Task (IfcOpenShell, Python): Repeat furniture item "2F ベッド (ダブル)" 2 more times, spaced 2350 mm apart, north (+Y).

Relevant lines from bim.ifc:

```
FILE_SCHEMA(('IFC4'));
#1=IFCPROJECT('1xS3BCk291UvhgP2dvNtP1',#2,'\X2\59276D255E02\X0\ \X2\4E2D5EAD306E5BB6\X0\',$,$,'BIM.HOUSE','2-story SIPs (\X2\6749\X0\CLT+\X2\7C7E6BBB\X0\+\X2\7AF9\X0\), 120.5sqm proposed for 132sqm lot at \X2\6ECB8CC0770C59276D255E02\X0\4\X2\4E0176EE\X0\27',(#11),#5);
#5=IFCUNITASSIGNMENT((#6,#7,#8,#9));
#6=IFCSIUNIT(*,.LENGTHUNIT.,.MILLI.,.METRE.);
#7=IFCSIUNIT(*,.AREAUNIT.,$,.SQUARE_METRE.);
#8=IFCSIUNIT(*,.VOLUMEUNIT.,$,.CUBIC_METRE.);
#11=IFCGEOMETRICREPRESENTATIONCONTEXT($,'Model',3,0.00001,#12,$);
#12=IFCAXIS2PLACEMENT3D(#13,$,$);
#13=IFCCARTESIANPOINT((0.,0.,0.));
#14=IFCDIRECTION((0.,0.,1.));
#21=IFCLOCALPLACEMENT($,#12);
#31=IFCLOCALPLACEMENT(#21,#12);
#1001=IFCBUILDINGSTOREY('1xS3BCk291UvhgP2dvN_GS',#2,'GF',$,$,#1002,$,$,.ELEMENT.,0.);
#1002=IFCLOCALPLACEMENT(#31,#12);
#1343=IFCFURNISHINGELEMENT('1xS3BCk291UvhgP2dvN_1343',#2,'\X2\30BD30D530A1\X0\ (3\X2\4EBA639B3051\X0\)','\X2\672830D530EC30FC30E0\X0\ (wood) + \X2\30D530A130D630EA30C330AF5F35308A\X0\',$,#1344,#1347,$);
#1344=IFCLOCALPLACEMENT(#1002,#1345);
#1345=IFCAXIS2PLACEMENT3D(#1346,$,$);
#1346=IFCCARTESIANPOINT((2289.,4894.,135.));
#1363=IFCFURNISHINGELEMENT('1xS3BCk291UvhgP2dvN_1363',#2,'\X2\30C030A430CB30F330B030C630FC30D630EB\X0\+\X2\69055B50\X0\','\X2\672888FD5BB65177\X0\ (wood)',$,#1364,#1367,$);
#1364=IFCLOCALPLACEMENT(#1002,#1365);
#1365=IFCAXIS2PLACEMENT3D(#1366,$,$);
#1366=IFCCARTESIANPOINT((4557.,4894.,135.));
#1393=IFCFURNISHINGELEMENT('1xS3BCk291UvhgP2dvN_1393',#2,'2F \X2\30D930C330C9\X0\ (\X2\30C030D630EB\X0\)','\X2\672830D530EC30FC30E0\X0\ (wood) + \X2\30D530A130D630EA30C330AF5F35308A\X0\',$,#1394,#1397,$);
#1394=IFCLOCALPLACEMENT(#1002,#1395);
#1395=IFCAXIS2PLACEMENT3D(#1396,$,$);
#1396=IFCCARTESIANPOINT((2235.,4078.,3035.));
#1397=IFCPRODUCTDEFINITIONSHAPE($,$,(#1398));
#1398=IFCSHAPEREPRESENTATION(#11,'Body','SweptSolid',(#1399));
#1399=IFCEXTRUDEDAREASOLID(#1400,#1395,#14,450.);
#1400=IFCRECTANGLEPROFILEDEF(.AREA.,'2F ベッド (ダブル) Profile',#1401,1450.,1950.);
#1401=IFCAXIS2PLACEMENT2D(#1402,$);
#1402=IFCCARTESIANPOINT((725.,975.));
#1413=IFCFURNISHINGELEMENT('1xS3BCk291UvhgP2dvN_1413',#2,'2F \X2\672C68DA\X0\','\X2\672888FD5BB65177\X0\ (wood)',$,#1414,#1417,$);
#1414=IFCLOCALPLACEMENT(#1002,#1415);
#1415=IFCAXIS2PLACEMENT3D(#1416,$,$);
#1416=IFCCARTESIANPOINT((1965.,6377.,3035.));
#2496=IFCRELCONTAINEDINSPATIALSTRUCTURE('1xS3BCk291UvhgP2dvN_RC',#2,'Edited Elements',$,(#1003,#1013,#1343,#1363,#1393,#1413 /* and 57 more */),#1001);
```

```python
import numpy as np
import ifcopenshell
import ifcopenshell.api.geometry
import ifcopenshell.api.root
import ifcopenshell.util.element
import ifcopenshell.util.placement

model = ifcopenshell.open("bim.ifc")


def reuse_history(source, copy):
    """copy_class also copies each property set's owner history, people and application; keep the originals."""
    for rel in copy.IsDefinedBy:
        if rel.is_a("IfcRelDefinesByProperties") and (history := rel.RelatingPropertyDefinition.OwnerHistory):
            rel.RelatingPropertyDefinition.OwnerHistory = source.OwnerHistory
            ifcopenshell.util.element.remove_deep2(model, history)


source = model.by_id(1393)
base = ifcopenshell.util.placement.get_local_placement(source.ObjectPlacement)
step = np.array([0.0, 1.0, 0.0]) * 2350.0

for i in range(1, 3):
    copy = ifcopenshell.api.root.copy_class(model, product=source)
    copy.Representation = ifcopenshell.util.element.copy_deep(
        model, source.Representation, exclude=["IfcGeometricRepresentationContext", "IfcRepresentationMap"]
    )
    reuse_history(source, copy)
    matrix = base.copy()
    matrix[:3, 3] += i * step
    print("added at", matrix[:3, 3].round(3) + 0.0)
    ifcopenshell.api.geometry.edit_object_placement(model, product=copy, matrix=matrix, is_si=False)

model.write("bim_updated.ifc")
```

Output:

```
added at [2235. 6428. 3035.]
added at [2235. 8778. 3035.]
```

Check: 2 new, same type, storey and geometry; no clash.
